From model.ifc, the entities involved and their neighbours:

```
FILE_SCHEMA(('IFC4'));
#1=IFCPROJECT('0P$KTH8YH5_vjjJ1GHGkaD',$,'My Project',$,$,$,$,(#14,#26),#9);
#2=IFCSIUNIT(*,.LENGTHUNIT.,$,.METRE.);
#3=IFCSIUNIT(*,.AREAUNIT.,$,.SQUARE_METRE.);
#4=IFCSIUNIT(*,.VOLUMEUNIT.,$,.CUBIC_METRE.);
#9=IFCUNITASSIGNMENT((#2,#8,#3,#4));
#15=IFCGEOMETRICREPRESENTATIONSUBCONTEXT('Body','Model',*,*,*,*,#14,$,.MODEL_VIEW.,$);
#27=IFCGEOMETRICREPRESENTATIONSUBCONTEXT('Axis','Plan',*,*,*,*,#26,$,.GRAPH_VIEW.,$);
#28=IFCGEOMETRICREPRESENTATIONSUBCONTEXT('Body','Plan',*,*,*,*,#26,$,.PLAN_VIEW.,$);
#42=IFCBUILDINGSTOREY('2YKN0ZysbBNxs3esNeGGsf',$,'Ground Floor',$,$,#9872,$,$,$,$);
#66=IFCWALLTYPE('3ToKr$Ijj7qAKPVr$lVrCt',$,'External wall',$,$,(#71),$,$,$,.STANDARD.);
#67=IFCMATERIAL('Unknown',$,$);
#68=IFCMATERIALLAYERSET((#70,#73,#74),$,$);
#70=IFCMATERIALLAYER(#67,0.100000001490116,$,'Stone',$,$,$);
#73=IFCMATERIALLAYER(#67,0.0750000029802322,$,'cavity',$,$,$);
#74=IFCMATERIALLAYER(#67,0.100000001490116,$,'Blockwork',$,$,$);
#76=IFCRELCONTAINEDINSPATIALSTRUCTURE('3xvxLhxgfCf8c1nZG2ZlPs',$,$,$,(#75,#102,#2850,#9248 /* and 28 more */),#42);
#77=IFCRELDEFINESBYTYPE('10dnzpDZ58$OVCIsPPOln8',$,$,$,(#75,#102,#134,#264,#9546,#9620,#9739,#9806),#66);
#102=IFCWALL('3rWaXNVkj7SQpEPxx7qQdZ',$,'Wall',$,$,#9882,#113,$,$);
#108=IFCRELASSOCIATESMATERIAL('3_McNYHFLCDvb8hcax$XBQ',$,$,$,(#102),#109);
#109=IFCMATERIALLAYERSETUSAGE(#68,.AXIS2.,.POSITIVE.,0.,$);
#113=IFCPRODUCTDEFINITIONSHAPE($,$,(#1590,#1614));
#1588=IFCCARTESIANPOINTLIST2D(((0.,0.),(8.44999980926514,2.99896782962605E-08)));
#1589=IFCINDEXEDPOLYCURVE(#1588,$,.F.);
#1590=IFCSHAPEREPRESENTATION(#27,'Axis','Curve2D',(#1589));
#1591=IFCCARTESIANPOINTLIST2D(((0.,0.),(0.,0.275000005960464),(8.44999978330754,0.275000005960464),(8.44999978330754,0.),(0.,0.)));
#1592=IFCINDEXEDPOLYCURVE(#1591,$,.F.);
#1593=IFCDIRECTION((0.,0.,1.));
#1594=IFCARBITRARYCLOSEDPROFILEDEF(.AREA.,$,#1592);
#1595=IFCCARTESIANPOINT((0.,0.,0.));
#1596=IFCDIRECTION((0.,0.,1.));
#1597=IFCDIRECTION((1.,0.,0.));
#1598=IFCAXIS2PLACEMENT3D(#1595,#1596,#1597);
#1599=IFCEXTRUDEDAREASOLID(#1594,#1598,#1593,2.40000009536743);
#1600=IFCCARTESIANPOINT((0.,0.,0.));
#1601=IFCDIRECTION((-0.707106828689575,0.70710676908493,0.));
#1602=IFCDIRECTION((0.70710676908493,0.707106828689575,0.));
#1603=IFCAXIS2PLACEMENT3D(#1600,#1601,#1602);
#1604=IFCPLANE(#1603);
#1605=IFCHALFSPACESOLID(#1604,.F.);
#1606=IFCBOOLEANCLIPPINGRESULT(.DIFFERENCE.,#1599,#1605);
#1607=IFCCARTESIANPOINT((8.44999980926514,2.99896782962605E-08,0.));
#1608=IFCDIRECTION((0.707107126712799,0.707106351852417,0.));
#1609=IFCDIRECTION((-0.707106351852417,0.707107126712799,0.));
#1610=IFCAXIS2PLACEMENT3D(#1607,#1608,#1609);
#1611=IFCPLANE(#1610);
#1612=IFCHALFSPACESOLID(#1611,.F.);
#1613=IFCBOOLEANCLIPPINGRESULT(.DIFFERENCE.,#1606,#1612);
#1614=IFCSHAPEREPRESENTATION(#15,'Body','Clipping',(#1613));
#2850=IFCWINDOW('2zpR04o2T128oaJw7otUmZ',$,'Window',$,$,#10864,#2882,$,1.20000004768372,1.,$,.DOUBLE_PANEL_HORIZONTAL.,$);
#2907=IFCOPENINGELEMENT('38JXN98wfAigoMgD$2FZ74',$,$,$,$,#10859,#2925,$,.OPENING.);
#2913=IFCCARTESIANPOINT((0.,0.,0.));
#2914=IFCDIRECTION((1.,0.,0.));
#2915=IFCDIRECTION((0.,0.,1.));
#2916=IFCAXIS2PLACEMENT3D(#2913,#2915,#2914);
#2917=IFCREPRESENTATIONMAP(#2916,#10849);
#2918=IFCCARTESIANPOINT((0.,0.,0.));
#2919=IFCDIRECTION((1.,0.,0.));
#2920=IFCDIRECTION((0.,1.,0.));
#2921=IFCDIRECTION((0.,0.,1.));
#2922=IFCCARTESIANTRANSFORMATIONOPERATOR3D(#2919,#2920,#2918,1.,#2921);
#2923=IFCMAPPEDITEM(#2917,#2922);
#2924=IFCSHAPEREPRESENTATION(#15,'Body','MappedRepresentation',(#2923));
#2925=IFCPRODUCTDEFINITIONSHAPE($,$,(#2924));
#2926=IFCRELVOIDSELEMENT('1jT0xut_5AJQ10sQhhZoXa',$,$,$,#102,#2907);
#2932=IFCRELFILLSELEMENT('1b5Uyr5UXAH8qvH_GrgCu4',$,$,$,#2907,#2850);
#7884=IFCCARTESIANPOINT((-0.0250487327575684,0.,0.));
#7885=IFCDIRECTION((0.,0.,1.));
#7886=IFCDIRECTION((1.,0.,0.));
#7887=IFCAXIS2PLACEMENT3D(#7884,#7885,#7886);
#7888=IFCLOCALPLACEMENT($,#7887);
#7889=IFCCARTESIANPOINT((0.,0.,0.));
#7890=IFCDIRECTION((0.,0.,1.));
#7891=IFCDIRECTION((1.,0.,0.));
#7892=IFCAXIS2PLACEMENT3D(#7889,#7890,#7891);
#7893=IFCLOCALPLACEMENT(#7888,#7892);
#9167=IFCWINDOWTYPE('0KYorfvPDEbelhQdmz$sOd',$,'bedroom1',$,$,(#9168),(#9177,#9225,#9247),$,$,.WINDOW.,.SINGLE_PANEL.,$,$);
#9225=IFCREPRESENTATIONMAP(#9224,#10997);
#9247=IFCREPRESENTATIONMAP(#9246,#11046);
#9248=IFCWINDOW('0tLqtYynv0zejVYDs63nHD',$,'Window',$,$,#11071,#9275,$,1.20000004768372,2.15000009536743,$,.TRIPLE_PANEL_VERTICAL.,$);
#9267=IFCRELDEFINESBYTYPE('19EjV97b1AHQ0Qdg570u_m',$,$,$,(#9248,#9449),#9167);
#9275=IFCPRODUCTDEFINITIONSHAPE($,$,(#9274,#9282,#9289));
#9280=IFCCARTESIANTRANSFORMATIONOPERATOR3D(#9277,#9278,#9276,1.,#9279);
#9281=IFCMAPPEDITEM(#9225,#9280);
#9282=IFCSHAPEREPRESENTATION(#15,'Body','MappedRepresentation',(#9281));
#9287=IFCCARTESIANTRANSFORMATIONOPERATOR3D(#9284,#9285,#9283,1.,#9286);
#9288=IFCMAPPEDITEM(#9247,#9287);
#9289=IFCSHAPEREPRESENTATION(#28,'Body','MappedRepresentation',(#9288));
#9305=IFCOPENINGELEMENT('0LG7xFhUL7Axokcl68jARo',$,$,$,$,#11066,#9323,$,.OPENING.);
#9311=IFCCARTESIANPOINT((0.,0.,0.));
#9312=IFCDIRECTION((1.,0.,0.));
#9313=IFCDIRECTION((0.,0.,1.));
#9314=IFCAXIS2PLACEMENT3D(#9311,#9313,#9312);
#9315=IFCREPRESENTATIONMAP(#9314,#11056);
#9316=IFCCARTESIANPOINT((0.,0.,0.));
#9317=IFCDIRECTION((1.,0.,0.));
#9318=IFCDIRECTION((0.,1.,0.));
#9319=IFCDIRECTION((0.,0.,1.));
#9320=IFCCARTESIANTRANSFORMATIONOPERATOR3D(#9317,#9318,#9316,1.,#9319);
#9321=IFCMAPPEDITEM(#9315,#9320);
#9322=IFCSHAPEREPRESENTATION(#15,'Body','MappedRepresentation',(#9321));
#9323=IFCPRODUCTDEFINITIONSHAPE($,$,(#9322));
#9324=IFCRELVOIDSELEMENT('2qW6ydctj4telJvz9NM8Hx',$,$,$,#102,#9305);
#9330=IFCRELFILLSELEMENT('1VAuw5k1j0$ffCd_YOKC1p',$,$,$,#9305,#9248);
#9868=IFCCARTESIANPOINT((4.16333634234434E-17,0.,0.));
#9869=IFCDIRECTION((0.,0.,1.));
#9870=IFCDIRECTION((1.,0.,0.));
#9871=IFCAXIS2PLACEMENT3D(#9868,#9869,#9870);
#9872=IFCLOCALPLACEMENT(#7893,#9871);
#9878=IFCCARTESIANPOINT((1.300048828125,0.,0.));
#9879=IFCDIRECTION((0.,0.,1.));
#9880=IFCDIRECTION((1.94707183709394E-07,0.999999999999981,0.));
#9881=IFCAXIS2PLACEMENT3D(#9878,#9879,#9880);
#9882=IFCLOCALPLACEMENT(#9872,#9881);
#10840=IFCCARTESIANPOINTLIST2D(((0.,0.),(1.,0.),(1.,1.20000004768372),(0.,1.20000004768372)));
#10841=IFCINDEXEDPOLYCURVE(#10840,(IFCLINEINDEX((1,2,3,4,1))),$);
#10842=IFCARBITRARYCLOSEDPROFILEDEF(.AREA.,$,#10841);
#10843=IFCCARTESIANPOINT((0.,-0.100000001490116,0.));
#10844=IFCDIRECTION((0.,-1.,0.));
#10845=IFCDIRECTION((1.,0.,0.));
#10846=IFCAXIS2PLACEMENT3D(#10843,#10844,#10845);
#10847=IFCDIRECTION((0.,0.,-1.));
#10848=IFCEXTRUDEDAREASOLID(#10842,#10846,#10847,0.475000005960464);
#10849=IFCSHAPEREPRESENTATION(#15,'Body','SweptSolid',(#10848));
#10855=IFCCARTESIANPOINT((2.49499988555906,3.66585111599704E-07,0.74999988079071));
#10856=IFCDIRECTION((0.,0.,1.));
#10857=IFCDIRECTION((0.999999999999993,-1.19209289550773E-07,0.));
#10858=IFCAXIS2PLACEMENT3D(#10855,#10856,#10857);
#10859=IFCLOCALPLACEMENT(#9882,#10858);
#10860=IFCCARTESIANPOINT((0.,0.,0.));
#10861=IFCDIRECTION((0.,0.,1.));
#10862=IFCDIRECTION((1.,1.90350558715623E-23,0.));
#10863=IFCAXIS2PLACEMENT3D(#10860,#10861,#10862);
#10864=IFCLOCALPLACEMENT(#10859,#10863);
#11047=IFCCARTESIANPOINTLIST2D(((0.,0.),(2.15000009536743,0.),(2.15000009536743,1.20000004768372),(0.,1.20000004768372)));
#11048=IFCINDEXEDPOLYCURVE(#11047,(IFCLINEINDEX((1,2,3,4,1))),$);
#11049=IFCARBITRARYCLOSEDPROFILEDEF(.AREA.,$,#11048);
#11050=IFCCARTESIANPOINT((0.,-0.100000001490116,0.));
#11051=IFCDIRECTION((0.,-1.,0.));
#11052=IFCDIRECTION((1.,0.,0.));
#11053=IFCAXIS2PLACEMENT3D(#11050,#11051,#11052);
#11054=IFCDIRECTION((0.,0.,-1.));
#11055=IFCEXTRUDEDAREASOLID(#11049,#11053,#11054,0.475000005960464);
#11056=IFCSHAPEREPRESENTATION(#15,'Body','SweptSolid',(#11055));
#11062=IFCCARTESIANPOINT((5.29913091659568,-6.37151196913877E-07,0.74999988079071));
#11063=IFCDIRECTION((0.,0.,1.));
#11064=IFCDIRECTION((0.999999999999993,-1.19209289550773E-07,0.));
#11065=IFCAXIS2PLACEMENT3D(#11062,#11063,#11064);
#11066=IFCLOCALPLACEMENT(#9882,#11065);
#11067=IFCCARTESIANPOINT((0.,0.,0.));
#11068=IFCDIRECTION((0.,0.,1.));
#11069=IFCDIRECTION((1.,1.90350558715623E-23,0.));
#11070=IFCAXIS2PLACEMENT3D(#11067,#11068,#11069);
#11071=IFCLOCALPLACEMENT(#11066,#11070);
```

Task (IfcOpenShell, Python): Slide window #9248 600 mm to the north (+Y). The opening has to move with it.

```python
import ifcopenshell
import ifcopenshell.api.geometry
import ifcopenshell.util.placement
import ifcopenshell.util.unit

model = ifcopenshell.open("model.ifc")
unit_scale = ifcopenshell.util.unit.calculate_unit_scale(model)

window = model.by_guid("0tLqtYynv0zejVYDs63nHD")
opening = window.FillsVoids[0].RelatingOpeningElement
wall = opening.VoidsElements[0].RelatingBuildingElement

wall_matrix = ifcopenshell.util.placement.get_local_placement(wall.ObjectPlacement)
shift = wall_matrix[:3, 0] * 0.6 / unit_scale
before = ifcopenshell.util.placement.get_local_placement(window.ObjectPlacement)[:3, 3].copy()

# The window is placed relative to its opening, so it follows when the opening moves.
matrix = ifcopenshell.util.placement.get_local_placement(opening.ObjectPlacement)
matrix[:3, 3] += shift
ifcopenshell.api.geometry.edit_object_placement(
    model, product=opening, matrix=matrix, is_si=False, should_transform_children=True
)

after = ifcopenshell.util.placement.get_local_placement(window.ObjectPlacement)[:3, 3]
print("window moved by", (after - before).round(3) + 0.0)

model.write("model_updated.ifc")
```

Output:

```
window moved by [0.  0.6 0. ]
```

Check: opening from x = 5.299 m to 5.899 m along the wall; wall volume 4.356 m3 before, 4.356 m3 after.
